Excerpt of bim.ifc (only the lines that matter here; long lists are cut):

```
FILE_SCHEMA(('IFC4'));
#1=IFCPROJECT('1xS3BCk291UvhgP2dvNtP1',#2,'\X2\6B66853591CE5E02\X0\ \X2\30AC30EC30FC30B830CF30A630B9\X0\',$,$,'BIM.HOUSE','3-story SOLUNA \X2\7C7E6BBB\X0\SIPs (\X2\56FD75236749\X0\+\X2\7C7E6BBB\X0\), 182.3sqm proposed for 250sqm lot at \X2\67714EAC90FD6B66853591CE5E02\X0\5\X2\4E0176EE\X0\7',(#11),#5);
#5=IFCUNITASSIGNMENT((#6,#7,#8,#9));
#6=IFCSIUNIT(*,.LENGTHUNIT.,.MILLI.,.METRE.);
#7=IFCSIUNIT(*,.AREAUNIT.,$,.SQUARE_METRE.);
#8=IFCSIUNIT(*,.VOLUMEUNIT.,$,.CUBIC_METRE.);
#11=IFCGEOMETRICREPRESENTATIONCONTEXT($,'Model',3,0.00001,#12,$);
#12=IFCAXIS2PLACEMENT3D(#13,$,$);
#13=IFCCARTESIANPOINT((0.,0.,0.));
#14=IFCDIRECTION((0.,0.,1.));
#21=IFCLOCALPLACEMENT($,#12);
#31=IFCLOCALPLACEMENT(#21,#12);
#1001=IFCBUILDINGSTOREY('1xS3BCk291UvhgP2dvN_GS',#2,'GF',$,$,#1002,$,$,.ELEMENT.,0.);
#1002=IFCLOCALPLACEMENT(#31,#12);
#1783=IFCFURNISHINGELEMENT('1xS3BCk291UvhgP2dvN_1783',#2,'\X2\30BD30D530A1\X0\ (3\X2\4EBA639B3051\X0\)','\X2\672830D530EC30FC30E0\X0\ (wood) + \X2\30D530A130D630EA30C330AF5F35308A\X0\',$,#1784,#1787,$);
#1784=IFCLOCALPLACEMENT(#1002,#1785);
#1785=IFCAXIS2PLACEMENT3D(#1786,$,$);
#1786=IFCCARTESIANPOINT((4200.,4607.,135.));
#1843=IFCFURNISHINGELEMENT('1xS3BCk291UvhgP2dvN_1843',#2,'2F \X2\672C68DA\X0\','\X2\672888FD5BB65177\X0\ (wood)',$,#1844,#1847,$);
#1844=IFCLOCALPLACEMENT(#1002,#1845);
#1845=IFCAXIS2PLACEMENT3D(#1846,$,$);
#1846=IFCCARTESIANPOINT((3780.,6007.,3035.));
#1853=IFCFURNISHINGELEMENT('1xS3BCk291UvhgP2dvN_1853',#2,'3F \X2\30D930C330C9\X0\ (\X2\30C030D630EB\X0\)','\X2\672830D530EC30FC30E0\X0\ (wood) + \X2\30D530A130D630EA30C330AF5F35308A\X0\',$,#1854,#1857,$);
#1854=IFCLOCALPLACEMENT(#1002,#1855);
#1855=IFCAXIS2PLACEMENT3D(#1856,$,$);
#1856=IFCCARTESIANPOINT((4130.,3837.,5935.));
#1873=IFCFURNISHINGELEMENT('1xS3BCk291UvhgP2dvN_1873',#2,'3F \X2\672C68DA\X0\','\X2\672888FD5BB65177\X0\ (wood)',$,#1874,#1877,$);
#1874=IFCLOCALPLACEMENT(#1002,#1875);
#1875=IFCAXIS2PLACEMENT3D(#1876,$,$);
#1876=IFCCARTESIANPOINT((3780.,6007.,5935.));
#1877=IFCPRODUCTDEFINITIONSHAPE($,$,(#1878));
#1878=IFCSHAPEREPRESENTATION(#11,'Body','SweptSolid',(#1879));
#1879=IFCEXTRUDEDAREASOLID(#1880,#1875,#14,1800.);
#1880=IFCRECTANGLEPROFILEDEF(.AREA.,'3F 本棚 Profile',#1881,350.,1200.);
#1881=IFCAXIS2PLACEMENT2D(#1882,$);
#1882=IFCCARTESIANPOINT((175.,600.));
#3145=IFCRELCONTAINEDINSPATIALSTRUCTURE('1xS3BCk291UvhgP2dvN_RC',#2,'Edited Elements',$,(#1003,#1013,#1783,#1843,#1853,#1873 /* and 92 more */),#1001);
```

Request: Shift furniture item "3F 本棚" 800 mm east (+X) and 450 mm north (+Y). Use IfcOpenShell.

```python
import ifcopenshell
import ifcopenshell.api.geometry
import ifcopenshell.util.placement
import ifcopenshell.util.unit

model = ifcopenshell.open("bim.ifc")
unit_scale = ifcopenshell.util.unit.calculate_unit_scale(model)

item = model.by_guid("1xS3BCk291UvhgP2dvN_1873")
matrix = ifcopenshell.util.placement.get_local_placement(item.ObjectPlacement)
matrix[0, 3] += 0.8 / unit_scale
matrix[1, 3] += 0.45 / unit_scale
ifcopenshell.api.geometry.edit_object_placement(model, product=item, matrix=matrix, is_si=False)

print(ifcopenshell.util.placement.get_local_placement(item.ObjectPlacement).round(3) + 0.0)

model.write("bim_updated.ifc")
```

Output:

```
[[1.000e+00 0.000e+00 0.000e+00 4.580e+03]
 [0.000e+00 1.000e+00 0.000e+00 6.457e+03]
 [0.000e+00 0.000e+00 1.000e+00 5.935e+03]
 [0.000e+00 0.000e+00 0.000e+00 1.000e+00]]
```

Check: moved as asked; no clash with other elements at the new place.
